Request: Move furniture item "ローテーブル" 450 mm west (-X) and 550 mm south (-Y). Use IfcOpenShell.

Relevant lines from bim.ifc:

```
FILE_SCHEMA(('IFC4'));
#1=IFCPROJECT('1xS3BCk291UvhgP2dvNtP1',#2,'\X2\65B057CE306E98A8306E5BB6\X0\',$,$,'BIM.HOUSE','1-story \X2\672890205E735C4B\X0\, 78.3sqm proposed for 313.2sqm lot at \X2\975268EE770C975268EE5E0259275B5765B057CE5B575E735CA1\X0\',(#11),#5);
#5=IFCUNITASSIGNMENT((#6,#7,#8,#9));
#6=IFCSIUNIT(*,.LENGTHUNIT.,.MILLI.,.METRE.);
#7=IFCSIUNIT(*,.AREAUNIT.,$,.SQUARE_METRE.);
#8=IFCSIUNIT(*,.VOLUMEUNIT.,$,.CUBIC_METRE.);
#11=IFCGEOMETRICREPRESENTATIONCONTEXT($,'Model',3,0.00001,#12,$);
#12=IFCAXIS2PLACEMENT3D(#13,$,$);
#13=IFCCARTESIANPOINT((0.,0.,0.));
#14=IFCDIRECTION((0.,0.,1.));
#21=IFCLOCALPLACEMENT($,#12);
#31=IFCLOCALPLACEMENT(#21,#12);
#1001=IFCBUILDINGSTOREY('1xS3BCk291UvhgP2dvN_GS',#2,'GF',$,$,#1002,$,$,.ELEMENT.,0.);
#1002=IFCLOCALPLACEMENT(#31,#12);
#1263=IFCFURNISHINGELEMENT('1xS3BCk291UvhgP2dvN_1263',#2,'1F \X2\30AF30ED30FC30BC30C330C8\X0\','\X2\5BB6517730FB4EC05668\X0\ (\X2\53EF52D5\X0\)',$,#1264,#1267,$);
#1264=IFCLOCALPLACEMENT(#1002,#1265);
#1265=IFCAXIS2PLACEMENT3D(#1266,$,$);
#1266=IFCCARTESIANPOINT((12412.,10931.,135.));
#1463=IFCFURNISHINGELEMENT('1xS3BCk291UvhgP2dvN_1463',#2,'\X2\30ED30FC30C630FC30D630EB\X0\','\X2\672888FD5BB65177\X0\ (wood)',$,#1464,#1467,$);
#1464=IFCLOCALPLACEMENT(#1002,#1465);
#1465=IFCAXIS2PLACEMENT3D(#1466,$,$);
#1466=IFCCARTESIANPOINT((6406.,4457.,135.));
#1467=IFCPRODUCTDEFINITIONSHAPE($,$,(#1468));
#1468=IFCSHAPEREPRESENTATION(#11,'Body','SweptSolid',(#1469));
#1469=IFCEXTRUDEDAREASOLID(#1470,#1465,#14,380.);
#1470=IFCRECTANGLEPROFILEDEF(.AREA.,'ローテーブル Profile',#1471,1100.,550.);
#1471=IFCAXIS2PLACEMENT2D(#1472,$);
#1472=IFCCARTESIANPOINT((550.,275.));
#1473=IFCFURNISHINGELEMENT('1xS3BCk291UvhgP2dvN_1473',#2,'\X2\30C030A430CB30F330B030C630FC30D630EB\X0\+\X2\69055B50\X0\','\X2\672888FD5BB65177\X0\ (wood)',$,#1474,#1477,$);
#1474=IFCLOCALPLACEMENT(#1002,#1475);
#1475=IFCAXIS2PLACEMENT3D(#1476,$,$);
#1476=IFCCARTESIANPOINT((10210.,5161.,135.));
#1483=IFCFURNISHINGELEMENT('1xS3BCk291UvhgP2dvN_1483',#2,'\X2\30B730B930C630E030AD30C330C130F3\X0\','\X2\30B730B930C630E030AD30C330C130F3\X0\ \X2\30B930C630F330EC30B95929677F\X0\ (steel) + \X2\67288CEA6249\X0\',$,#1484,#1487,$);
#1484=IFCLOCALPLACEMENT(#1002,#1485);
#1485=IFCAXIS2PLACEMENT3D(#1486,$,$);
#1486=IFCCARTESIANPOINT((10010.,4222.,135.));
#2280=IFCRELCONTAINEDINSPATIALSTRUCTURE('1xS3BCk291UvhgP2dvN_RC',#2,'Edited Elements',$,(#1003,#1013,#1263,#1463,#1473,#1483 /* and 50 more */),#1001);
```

```python
import ifcopenshell
import ifcopenshell.api.geometry
import ifcopenshell.util.placement

model = ifcopenshell.open("bim.ifc")

item = model.by_guid("1xS3BCk291UvhgP2dvN_1463")
matrix = ifcopenshell.util.placement.get_local_placement(item.ObjectPlacement)
matrix[0, 3] -= 450.0
matrix[1, 3] -= 550.0
ifcopenshell.api.geometry.edit_object_placement(model, product=item, matrix=matrix, is_si=False)

print(ifcopenshell.util.placement.get_local_placement(item.ObjectPlacement).round(3) + 0.0)

model.write("bim-out.ifc")
```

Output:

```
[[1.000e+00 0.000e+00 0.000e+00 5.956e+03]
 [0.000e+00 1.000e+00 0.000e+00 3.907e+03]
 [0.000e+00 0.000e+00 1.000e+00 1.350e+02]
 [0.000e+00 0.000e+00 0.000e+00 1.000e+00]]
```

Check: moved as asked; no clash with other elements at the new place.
